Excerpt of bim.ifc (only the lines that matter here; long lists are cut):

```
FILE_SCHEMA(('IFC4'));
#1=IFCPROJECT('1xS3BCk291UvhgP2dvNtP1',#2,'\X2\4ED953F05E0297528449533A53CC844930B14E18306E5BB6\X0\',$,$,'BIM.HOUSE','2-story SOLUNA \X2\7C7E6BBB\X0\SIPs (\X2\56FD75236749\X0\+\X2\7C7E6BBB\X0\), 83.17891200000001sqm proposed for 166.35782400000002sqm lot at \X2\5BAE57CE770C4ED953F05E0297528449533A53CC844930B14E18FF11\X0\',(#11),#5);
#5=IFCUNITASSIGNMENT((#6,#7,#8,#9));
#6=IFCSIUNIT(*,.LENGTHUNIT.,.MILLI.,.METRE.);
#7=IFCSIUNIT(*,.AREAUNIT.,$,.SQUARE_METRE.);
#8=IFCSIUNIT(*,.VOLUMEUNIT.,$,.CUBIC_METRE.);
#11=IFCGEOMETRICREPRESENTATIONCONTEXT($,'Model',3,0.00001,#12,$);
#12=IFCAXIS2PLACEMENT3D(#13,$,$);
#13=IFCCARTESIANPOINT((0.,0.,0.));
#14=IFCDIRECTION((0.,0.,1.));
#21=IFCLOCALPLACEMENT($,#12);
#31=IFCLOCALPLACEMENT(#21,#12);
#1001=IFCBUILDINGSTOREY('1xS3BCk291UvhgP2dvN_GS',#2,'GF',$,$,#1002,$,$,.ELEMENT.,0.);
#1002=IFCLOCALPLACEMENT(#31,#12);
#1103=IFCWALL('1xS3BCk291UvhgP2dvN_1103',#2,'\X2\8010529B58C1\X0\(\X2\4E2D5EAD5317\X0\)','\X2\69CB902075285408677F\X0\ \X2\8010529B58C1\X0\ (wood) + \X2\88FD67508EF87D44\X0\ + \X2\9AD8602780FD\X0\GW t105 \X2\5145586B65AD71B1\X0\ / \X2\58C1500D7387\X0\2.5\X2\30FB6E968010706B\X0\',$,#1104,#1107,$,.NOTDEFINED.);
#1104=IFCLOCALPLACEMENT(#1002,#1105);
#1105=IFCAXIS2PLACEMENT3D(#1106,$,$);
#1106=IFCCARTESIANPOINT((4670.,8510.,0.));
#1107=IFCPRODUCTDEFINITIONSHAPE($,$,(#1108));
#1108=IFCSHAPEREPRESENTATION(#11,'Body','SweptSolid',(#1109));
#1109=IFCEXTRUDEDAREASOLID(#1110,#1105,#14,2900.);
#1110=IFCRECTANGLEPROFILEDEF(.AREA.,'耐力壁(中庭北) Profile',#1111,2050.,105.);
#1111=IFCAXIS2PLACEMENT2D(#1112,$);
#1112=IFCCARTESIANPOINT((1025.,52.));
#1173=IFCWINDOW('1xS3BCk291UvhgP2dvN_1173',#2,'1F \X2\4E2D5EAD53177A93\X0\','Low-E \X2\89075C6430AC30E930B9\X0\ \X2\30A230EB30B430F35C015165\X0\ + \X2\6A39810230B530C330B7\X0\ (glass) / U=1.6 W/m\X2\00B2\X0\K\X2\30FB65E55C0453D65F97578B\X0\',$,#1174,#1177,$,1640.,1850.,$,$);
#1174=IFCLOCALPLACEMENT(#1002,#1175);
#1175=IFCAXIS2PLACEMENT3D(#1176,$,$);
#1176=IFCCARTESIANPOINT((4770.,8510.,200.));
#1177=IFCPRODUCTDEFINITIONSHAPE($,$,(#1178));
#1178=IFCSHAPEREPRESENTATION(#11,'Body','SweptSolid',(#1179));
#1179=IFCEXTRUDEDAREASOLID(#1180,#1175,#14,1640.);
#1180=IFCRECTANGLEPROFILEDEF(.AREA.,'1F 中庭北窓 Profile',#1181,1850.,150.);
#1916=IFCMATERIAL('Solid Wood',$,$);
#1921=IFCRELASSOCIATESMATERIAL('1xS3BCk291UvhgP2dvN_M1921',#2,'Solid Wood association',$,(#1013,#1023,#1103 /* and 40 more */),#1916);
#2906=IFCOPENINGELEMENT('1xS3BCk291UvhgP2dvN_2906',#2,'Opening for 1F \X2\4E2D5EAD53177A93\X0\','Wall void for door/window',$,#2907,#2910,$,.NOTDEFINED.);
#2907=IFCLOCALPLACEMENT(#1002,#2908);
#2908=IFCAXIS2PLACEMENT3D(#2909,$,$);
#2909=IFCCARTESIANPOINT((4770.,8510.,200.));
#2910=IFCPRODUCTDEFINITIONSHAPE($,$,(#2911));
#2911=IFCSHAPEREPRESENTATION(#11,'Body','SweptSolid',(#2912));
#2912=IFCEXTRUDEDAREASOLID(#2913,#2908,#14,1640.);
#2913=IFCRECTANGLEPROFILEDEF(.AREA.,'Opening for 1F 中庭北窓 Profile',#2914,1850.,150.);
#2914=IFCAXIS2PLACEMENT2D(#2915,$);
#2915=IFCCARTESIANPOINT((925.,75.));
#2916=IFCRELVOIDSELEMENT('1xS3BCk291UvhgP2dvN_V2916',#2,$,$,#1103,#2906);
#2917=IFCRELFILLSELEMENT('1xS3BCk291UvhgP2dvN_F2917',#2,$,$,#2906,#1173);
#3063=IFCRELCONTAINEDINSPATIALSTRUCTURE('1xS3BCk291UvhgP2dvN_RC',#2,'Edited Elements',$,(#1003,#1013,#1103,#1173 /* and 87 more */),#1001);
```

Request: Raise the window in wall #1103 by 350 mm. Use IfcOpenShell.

```python
import numpy as np
import ifcopenshell
import ifcopenshell.api.geometry
import ifcopenshell.util.placement
import ifcopenshell.util.unit

model = ifcopenshell.open("bim.ifc")
unit_scale = ifcopenshell.util.unit.calculate_unit_scale(model)

window = model.by_guid("1xS3BCk291UvhgP2dvN_1173")
opening = window.FillsVoids[0].RelatingOpeningElement
dz = 350.0

shift = np.array([0.0, 0.0, dz])
# The window is not placed relative to its opening, so move both.
for product in (opening, window):
    matrix = ifcopenshell.util.placement.get_local_placement(product.ObjectPlacement)
    matrix[:3, 3] += shift
    ifcopenshell.api.geometry.edit_object_placement(model, product=product, matrix=matrix, is_si=False)

print(f"moved by {dz * unit_scale:+.3f} m")

model.write("bim_v2.ifc")
```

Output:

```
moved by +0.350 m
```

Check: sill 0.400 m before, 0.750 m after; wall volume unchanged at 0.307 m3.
